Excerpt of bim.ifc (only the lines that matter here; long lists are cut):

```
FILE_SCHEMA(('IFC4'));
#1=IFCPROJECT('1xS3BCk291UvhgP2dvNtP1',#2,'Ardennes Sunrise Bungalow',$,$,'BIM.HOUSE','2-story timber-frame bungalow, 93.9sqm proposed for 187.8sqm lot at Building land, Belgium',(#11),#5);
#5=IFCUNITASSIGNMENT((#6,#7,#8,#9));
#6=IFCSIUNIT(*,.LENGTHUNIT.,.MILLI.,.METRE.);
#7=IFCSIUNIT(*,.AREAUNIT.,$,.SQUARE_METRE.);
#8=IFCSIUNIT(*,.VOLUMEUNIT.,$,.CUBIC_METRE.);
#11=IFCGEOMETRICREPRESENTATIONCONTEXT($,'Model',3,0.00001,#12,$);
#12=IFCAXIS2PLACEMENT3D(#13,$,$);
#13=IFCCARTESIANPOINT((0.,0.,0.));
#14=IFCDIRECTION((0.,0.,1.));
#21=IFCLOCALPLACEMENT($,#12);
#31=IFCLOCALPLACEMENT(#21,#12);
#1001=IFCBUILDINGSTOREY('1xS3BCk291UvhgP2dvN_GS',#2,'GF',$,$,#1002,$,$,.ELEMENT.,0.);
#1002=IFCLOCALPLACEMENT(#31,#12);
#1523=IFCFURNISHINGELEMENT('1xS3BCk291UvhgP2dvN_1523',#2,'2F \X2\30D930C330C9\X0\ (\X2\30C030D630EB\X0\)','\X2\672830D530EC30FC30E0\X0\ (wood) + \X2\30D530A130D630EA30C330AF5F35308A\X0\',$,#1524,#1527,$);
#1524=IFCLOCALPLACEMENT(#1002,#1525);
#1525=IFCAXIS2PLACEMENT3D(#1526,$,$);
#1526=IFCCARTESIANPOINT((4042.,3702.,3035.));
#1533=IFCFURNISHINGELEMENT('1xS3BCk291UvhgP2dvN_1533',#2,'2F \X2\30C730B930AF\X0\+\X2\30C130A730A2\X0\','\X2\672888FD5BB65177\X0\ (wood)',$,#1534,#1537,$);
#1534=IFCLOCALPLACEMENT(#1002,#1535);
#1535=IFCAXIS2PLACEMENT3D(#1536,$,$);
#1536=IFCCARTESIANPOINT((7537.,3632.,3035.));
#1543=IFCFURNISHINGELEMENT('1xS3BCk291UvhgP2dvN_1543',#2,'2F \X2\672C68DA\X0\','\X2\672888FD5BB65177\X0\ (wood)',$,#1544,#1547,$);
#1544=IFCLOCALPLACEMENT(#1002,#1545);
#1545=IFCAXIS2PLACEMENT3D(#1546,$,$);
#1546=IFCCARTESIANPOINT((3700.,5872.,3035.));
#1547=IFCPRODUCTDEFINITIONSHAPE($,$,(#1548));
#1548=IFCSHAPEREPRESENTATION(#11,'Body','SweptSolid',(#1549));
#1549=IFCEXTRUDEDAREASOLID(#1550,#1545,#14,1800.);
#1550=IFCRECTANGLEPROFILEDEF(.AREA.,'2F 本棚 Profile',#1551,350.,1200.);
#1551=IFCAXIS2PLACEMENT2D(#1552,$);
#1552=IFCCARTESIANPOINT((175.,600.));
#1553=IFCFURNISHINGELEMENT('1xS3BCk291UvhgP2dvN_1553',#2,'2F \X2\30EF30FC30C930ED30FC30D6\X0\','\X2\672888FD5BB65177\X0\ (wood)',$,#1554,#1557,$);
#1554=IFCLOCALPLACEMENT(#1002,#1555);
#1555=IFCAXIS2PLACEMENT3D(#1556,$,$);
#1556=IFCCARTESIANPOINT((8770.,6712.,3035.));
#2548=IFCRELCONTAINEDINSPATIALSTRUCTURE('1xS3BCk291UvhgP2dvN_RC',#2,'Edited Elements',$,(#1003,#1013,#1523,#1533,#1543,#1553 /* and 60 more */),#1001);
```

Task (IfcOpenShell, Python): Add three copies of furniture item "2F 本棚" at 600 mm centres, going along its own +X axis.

```python
import ifcopenshell
import ifcopenshell.api.geometry
import ifcopenshell.api.root
import ifcopenshell.util.element
import ifcopenshell.util.placement

model = ifcopenshell.open("bim.ifc")


def reuse_history(source, copy):
    """copy_class also copies each property set's owner history, people and application; keep the originals."""
    for rel in copy.IsDefinedBy:
        if rel.is_a("IfcRelDefinesByProperties") and (history := rel.RelatingPropertyDefinition.OwnerHistory):
            rel.RelatingPropertyDefinition.OwnerHistory = source.OwnerHistory
            ifcopenshell.util.element.remove_deep2(model, history)


source = model.by_id(1543)
base = ifcopenshell.util.placement.get_local_placement(source.ObjectPlacement)
step = base[:3, 0] * 600.0

for i in range(1, 4):
    copy = ifcopenshell.api.root.copy_class(model, product=source)
    copy.Representation = ifcopenshell.util.element.copy_deep(
        model, source.Representation, exclude=["IfcGeometricRepresentationContext", "IfcRepresentationMap"]
    )
    reuse_history(source, copy)
    matrix = base.copy()
    matrix[:3, 3] += i * step
    print("added at", matrix[:3, 3].round(3) + 0.0)
    ifcopenshell.api.geometry.edit_object_placement(model, product=copy, matrix=matrix, is_si=False)

model.write("bim_v2.ifc")
```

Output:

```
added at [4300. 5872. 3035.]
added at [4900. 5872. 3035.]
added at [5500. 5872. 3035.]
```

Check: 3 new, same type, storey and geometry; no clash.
